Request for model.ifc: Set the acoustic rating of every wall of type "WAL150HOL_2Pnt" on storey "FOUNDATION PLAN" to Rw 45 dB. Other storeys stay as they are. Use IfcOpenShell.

First a look at what the model holds.

```python
import ifcopenshell
import ifcopenshell.util.element

model = ifcopenshell.open("model.ifc")
print(model.schema)
storey = next(s for s in model.by_type("IfcBuildingStorey") if s.Name == "FOUNDATION PLAN")
walls = [e for e in ifcopenshell.util.element.get_decomposition(storey) if e.is_a("IfcWall")]
seen = {}
for e in walls:
    element_type = ifcopenshell.util.element.get_type(e)
    key = (element_type.Name if element_type != e and element_type else None, ifcopenshell.util.element.get_pset(e, "Pset_WallCommon", "AcousticRating"))
    seen[key] = seen.get(key, 0) + 1
for (name, value), count in sorted(seen.items(), key=str):
    print(count, "x", name, "|", value)
```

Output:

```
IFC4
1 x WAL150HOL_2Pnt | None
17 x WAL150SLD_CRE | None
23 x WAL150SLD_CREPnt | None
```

```python
import ifcopenshell
import ifcopenshell.api.pset
import ifcopenshell.util.element

model = ifcopenshell.open("model.ifc")

storey = next(s for s in model.by_type("IfcBuildingStorey") if s.Name == "FOUNDATION PLAN")
walls = [e for e in ifcopenshell.util.element.get_decomposition(storey) if e.is_a("IfcWall")]

count = 0
for e in walls:
    element_type = ifcopenshell.util.element.get_type(e)
    if element_type in (None, e) or element_type.Name != "WAL150HOL_2Pnt":
        continue
    # add_pset returns the element's existing set when there is one.
    pset = ifcopenshell.api.pset.add_pset(model, product=e, name="Pset_WallCommon")
    ifcopenshell.api.pset.edit_pset(model, pset=pset, properties={"AcousticRating": "Rw 45 dB"})
    count += 1

print(count, "walls updated")

model.write("model_v2.ifc")
```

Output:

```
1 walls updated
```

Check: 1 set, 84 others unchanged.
